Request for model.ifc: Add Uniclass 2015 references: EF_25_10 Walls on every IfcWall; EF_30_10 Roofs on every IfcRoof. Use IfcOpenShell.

First a look at what the model holds.

```python
import ifcopenshell

model = ifcopenshell.open("model.ifc")
print(model.schema)
print("classifications:", [c.Name for c in model.by_type("IfcClassification")])
for ifc_class in ("IfcDoor", "IfcRoof", "IfcStair", "IfcWall", "IfcWindow"):
    print(ifc_class, len(model.by_type(ifc_class)))
```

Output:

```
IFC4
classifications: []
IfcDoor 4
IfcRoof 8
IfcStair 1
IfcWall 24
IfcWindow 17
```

```python
import ifcopenshell
import ifcopenshell.api.classification

model = ifcopenshell.open("model.ifc")

system = ifcopenshell.api.classification.add_classification(model, classification="Uniclass 2015")

codes = {
    "IfcWall": ("EF_25_10", "Walls"),
    "IfcRoof": ("EF_30_10", "Roofs"),
}
for ifc_class, (code, name) in codes.items():
    products = model.by_type(ifc_class)
    ifcopenshell.api.classification.add_reference(
        model, products=products, classification=system, identification=code, name=name
    )
    print(code, len(products))

model.write("model_rev.ifc")
```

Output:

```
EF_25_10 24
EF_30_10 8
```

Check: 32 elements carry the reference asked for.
